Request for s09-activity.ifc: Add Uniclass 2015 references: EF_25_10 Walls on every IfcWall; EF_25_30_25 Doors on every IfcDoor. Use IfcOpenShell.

First a look at what the model holds.

```python
import ifcopenshell

model = ifcopenshell.open("s09-activity.ifc")
print(model.schema)
print("classifications:", [c.Name for c in model.by_type("IfcClassification")])
for ifc_class in ("IfcDoor", "IfcRoof", "IfcStair", "IfcWall", "IfcWindow"):
    print(ifc_class, len(model.by_type(ifc_class)))
```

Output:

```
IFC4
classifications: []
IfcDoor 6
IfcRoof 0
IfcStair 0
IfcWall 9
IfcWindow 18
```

```python
import ifcopenshell
import ifcopenshell.api.classification

model = ifcopenshell.open("s09-activity.ifc")

system = ifcopenshell.api.classification.add_classification(model, classification="Uniclass 2015")

codes = {
    "IfcWall": ("EF_25_10", "Walls"),
    "IfcDoor": ("EF_25_30_25", "Doors"),
}
for ifc_class, (code, name) in codes.items():
    products = model.by_type(ifc_class)
    ifcopenshell.api.classification.add_reference(
        model, products=products, classification=system, identification=code, name=name
    )
    print(code, len(products))

model.write("s09-activity_rev.ifc")
```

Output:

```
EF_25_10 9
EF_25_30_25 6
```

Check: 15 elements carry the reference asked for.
